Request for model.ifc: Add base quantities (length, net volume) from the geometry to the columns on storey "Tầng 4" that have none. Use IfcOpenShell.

First a look at what the model holds.

```python
import ifcopenshell
import ifcopenshell.util.element
import ifcopenshell.util.unit

model = ifcopenshell.open("model.ifc")
print(model.schema)
for unit_type in ("LENGTHUNIT", "AREAUNIT", "VOLUMEUNIT"):
    print(unit_type, ifcopenshell.util.unit.calculate_unit_scale(model, unit_type))
storey = next(s for s in model.by_type("IfcBuildingStorey") if s.Name == "Tầng 4")
columns = [e for e in ifcopenshell.util.element.get_decomposition(storey) if e.is_a("IfcColumn")]
for e in sorted(columns, key=lambda e: e.id()):
    print(e.id(), e.is_a(), e.Name, list(ifcopenshell.util.element.get_psets(e, qtos_only=True)), sep=" | ")
```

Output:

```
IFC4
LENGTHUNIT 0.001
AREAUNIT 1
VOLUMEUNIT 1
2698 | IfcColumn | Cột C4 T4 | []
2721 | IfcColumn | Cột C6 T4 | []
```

```python
import ifcopenshell
import ifcopenshell.api.pset
import ifcopenshell.geom
import ifcopenshell.util.element
import ifcopenshell.util.shape
import ifcopenshell.util.unit

model = ifcopenshell.open("model.ifc")
unit_scale = ifcopenshell.util.unit.calculate_unit_scale(model)
volume_scale = ifcopenshell.util.unit.calculate_unit_scale(model, "VOLUMEUNIT")
settings = ifcopenshell.geom.settings()

storey = next(s for s in model.by_type("IfcBuildingStorey") if s.Name == "Tầng 4")
columns = [e for e in ifcopenshell.util.element.get_decomposition(storey) if e.is_a("IfcColumn")]

for e in sorted(columns, key=lambda e: e.id()):
    if ifcopenshell.util.element.get_psets(e, qtos_only=True, should_inherit=False):
        continue
    # Geometry comes back in metres, in the element's own axes.
    shape = ifcopenshell.geom.create_shape(settings, e)
    values = {
        "Length": ifcopenshell.util.shape.get_z(shape.geometry) / unit_scale,
        "NetVolume": ifcopenshell.util.shape.get_volume(shape.geometry) / volume_scale,
    }
    qto = ifcopenshell.api.pset.add_qto(model, product=e, name="Qto_ColumnBaseQuantities")
    ifcopenshell.api.pset.edit_qto(model, qto=qto, properties=values)
    print(e.id(), {k: round(v, 3) for k, v in values.items()})

model.write("model_edited.ifc")
```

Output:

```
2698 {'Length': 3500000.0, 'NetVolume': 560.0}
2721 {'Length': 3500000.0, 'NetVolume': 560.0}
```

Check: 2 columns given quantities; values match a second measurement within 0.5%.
